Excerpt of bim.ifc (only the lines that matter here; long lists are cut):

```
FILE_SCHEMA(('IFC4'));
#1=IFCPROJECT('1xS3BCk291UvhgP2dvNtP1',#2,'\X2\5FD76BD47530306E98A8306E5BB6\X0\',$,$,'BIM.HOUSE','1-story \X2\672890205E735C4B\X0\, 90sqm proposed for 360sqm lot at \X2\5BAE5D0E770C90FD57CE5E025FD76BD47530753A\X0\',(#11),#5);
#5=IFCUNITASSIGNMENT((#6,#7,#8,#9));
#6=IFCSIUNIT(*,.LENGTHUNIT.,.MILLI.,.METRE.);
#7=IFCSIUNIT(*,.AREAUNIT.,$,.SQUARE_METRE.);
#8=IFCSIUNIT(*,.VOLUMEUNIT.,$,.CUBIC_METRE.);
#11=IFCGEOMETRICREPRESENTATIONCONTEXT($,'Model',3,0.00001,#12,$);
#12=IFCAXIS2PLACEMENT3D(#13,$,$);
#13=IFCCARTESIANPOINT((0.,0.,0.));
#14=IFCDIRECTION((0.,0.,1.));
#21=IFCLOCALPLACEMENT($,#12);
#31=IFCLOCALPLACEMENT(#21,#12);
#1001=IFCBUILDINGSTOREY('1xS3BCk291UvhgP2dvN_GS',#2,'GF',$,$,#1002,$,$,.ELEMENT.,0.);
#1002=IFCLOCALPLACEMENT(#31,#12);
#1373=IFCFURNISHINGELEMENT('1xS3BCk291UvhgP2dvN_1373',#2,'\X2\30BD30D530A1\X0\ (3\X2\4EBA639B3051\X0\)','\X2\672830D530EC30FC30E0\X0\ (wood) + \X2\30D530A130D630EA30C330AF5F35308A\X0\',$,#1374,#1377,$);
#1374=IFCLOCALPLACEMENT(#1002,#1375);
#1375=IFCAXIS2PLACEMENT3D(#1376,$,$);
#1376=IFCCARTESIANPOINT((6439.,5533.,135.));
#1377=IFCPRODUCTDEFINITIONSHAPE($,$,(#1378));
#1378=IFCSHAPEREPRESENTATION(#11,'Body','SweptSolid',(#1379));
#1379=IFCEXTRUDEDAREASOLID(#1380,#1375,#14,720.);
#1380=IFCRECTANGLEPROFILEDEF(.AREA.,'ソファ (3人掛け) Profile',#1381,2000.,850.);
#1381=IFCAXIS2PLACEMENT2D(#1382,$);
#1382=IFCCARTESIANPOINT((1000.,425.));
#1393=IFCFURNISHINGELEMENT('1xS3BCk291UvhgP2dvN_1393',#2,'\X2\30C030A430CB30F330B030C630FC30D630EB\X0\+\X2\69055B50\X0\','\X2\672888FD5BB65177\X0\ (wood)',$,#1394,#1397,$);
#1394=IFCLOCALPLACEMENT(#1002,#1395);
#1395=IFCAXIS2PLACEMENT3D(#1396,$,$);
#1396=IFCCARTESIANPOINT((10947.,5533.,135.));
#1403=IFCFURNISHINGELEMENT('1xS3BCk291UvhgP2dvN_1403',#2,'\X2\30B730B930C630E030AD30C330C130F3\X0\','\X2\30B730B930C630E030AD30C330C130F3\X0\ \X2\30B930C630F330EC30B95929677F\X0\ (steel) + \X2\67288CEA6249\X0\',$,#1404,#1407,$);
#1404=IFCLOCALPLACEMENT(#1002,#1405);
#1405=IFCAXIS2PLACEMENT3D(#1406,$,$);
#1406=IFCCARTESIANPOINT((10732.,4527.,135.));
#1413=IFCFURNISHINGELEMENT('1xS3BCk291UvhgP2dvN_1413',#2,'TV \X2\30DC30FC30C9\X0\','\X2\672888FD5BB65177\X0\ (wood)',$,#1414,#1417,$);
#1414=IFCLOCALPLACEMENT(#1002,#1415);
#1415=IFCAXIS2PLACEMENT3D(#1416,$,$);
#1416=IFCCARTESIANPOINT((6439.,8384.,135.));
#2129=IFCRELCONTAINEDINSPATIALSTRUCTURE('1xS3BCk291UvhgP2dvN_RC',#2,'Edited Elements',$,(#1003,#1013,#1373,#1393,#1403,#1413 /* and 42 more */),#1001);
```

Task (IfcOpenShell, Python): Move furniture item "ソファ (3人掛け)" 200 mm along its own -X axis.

```python
import ifcopenshell
import ifcopenshell.api.geometry
import ifcopenshell.util.placement
import ifcopenshell.util.unit

model = ifcopenshell.open("bim.ifc")
unit_scale = ifcopenshell.util.unit.calculate_unit_scale(model)

item = model.by_guid("1xS3BCk291UvhgP2dvN_1373")
matrix = ifcopenshell.util.placement.get_local_placement(item.ObjectPlacement)
matrix[:3, 3] -= matrix[:3, 0] * 0.2 / unit_scale
ifcopenshell.api.geometry.edit_object_placement(model, product=item, matrix=matrix, is_si=False)

print(ifcopenshell.util.placement.get_local_placement(item.ObjectPlacement).round(3) + 0.0)

model.write("bim-out.ifc")
```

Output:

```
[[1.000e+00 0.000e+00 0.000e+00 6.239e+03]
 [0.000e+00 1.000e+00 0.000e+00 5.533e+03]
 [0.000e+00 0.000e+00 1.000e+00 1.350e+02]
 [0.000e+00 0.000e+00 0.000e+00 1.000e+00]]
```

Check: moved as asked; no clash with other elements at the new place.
